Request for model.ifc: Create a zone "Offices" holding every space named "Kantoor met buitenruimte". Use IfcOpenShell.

First a look at what the model holds.

```python
import ifcopenshell

model = ifcopenshell.open("model.ifc")
print(model.schema)
seen = {}
for space in model.by_type("IfcSpace"):
    seen[space.LongName] = seen.get(space.LongName, 0) + 1
for name, count in sorted(seen.items(), key=str):
    print(count, "x", name)
print("zones:", [z.Name for z in model.by_type("IfcZone")][:20])
```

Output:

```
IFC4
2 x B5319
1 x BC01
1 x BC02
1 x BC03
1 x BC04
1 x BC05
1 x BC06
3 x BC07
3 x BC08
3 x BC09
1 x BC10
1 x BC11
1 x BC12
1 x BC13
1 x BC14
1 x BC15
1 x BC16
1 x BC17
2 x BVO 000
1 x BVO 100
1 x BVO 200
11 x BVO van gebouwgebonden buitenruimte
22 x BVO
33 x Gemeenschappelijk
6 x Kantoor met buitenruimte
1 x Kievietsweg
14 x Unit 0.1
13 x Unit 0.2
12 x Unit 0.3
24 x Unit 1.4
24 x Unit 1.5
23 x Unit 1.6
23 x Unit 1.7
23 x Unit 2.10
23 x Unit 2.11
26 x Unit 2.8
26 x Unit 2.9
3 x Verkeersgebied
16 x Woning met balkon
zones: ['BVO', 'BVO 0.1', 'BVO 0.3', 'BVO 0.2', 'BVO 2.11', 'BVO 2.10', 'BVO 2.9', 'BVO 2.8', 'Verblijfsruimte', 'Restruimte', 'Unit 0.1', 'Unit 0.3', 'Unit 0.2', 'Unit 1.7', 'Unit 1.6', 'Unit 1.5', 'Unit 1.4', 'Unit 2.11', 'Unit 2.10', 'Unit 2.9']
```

```python
import ifcopenshell
import ifcopenshell.api.group
import ifcopenshell.api.root

model = ifcopenshell.open("model.ifc")

names = {"Kantoor met buitenruimte"}
spaces = [s for s in model.by_type("IfcSpace") if s.LongName in names]

zone = ifcopenshell.api.root.create_entity(model, ifc_class="IfcZone", name="Offices")
ifcopenshell.api.group.assign_group(model, products=spaces, group=zone)
print(len(spaces), "spaces in", zone.Name)

model.write("model-out.ifc")
```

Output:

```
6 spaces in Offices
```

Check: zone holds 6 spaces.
